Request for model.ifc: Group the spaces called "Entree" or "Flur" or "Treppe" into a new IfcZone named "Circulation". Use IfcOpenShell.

First a look at what the model holds.

```python
import ifcopenshell

model = ifcopenshell.open("model.ifc")
print(model.schema)
seen = {}
for space in model.by_type("IfcSpace"):
    seen[space.LongName] = seen.get(space.LongName, 0) + 1
for name, count in sorted(seen.items(), key=str):
    print(count, "x", name)
print("zones:", [z.Name for z in model.by_type("IfcZone")][:20])
```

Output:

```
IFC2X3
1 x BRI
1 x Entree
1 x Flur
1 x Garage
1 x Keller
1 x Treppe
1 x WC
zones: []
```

```python
import ifcopenshell
import ifcopenshell.api.group
import ifcopenshell.api.root

model = ifcopenshell.open("model.ifc")

names = {"Entree", "Flur", "Treppe"}
spaces = [s for s in model.by_type("IfcSpace") if s.LongName in names]

zone = ifcopenshell.api.root.create_entity(model, ifc_class="IfcZone", name="Circulation")
ifcopenshell.api.group.assign_group(model, products=spaces, group=zone)
print(len(spaces), "spaces in", zone.Name)

model.write("model_updated.ifc")
```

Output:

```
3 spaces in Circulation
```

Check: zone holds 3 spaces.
